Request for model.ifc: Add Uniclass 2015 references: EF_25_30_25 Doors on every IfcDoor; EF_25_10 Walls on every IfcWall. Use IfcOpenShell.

First a look at what the model holds.

```python
import ifcopenshell

model = ifcopenshell.open("model.ifc")
print(model.schema)
print("classifications:", [c.Name for c in model.by_type("IfcClassification")])
for ifc_class in ("IfcDoor", "IfcRoof", "IfcStair", "IfcWall", "IfcWindow"):
    print(ifc_class, len(model.by_type(ifc_class)))
```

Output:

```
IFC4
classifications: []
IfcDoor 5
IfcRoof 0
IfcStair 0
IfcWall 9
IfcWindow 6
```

```python
import ifcopenshell
import ifcopenshell.api.classification

model = ifcopenshell.open("model.ifc")

system = ifcopenshell.api.classification.add_classification(model, classification="Uniclass 2015")

codes = {
    "IfcDoor": ("EF_25_30_25", "Doors"),
    "IfcWall": ("EF_25_10", "Walls"),
}
for ifc_class, (code, name) in codes.items():
    products = model.by_type(ifc_class)
    ifcopenshell.api.classification.add_reference(
        model, products=products, classification=system, identification=code, name=name
    )
    print(code, len(products))

model.write("model_v2.ifc")
```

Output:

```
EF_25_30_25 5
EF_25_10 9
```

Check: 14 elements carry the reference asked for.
